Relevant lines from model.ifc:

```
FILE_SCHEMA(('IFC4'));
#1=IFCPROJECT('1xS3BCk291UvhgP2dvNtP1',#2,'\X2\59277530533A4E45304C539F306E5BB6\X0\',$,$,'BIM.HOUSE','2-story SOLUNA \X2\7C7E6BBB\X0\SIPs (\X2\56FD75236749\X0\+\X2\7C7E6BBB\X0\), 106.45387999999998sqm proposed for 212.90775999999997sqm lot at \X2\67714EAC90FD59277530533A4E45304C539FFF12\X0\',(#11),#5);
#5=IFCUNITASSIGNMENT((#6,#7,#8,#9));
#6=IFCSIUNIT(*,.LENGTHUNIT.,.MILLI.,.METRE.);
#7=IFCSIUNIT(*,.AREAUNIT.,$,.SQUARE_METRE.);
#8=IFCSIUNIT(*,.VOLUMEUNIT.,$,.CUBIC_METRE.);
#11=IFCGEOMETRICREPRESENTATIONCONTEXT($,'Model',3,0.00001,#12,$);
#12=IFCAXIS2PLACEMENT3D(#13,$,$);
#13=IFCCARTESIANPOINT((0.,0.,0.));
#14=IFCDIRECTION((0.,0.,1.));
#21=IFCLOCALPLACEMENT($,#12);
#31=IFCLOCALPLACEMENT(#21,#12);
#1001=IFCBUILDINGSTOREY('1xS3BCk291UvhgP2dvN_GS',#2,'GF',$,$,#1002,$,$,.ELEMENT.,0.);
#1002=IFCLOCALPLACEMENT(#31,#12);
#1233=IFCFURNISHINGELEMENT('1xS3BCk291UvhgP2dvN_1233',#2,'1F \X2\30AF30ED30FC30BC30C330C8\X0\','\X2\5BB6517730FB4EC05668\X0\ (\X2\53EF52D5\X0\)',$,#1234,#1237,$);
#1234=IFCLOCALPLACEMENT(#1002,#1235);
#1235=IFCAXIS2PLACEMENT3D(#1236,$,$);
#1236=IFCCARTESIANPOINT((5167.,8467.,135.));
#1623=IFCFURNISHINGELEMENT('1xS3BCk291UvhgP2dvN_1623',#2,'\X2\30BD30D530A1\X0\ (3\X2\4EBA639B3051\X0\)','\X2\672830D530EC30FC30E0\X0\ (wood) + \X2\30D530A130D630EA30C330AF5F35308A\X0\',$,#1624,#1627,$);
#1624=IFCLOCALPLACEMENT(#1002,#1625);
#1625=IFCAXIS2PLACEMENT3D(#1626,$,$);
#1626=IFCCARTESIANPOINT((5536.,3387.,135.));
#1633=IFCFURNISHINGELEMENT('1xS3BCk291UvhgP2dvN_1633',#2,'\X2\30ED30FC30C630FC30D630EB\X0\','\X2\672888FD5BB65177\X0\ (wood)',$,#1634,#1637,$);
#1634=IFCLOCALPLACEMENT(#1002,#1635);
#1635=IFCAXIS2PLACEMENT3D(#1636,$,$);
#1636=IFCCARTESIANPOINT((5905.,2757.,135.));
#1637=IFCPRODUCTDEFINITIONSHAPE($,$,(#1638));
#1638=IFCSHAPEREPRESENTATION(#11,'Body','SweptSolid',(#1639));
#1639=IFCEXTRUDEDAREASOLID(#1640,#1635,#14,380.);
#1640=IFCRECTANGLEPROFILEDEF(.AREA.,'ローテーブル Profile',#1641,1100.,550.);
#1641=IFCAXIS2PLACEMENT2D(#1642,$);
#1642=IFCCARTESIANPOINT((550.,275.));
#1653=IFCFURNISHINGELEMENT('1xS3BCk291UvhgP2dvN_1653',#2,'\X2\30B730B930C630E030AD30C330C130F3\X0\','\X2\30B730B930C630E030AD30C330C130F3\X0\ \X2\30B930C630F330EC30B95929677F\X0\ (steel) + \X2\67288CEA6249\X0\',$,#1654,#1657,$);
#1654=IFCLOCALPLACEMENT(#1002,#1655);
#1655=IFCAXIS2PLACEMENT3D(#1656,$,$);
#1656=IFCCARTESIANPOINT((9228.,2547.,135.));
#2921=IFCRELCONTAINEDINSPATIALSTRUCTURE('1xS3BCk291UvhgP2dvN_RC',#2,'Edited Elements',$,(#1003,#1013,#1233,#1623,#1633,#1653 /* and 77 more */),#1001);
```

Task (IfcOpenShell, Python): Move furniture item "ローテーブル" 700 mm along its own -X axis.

```python
import ifcopenshell
import ifcopenshell.api.geometry
import ifcopenshell.util.placement
import ifcopenshell.util.unit

model = ifcopenshell.open("model.ifc")
unit_scale = ifcopenshell.util.unit.calculate_unit_scale(model)

item = model.by_guid("1xS3BCk291UvhgP2dvN_1633")
matrix = ifcopenshell.util.placement.get_local_placement(item.ObjectPlacement)
matrix[:3, 3] -= matrix[:3, 0] * 0.7 / unit_scale
ifcopenshell.api.geometry.edit_object_placement(model, product=item, matrix=matrix, is_si=False)

print(ifcopenshell.util.placement.get_local_placement(item.ObjectPlacement).round(3) + 0.0)

model.write("model_v2.ifc")
```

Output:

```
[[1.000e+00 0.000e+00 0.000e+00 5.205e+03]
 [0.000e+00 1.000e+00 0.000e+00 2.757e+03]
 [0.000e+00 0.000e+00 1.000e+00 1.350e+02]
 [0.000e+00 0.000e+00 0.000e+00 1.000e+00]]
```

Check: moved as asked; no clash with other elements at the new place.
